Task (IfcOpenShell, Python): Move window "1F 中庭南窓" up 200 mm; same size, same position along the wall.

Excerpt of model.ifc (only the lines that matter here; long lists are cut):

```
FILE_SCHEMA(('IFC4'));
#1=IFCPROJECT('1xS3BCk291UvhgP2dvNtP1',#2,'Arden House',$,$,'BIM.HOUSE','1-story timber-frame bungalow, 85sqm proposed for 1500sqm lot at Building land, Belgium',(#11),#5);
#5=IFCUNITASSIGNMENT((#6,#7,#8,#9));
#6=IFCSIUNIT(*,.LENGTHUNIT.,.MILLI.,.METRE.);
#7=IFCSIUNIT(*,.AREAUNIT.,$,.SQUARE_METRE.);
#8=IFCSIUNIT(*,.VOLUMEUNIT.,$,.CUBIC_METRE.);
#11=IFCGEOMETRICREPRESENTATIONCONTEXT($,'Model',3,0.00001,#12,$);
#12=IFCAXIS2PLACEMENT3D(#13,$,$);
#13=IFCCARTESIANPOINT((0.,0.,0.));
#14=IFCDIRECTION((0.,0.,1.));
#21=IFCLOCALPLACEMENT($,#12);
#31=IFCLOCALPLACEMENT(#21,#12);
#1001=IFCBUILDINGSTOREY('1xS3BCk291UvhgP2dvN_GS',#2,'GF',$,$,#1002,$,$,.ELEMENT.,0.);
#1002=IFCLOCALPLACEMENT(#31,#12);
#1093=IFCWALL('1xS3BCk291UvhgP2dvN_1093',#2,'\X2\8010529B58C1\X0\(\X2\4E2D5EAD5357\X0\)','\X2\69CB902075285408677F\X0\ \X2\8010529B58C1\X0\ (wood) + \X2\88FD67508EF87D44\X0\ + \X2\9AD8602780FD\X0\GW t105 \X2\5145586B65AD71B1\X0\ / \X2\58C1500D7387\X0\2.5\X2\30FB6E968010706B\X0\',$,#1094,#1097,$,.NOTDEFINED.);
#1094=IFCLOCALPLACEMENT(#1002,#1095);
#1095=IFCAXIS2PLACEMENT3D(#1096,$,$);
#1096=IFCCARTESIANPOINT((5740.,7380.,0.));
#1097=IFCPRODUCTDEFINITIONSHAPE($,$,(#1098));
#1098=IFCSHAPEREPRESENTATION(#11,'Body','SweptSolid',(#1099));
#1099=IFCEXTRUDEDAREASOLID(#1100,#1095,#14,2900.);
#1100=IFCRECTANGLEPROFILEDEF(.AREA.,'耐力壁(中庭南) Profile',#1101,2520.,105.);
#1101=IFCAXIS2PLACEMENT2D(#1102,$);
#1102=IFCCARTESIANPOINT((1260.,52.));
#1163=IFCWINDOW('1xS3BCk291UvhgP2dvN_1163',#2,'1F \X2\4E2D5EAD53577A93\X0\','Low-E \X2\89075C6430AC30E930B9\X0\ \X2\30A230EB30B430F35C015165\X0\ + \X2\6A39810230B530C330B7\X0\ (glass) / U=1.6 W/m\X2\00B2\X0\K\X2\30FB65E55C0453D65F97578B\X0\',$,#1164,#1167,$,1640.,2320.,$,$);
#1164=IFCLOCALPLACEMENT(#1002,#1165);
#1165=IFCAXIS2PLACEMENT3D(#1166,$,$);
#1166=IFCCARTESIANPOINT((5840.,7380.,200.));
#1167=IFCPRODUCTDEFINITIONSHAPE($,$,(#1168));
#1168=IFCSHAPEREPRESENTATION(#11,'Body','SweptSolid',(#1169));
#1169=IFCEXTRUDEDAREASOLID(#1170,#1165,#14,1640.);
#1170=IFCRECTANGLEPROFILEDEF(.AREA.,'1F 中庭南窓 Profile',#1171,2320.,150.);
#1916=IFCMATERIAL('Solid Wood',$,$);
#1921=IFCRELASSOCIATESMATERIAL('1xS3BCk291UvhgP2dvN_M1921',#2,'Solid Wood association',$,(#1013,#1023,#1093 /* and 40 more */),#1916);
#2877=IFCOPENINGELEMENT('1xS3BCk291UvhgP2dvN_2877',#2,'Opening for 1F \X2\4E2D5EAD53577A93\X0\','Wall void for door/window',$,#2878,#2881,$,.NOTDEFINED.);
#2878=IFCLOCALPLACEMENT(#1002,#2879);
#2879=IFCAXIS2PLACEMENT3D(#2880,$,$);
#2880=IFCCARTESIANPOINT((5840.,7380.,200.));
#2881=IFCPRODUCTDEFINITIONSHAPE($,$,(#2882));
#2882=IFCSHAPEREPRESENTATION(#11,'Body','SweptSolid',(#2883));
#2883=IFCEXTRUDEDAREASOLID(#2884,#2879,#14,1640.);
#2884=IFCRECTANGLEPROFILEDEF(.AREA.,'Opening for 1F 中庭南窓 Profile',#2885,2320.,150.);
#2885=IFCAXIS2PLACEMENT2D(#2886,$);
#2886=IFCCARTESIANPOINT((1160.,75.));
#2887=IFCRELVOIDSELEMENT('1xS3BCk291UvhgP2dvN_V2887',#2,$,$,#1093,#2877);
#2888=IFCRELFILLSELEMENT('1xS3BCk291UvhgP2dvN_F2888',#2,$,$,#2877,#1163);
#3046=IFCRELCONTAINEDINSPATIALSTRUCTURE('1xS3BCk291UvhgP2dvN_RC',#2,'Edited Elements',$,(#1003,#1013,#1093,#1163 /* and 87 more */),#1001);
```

```python
import numpy as np
import ifcopenshell
import ifcopenshell.api.geometry
import ifcopenshell.util.placement
import ifcopenshell.util.unit

model = ifcopenshell.open("model.ifc")
unit_scale = ifcopenshell.util.unit.calculate_unit_scale(model)

window = model.by_guid("1xS3BCk291UvhgP2dvN_1163")
opening = window.FillsVoids[0].RelatingOpeningElement
dz = 200.0

shift = np.array([0.0, 0.0, dz])
# The window is not placed relative to its opening, so move both.
for product in (opening, window):
    matrix = ifcopenshell.util.placement.get_local_placement(product.ObjectPlacement)
    matrix[:3, 3] += shift
    ifcopenshell.api.geometry.edit_object_placement(model, product=product, matrix=matrix, is_si=False)

print(f"moved by {dz * unit_scale:+.3f} m")

model.write("model-out.ifc")
```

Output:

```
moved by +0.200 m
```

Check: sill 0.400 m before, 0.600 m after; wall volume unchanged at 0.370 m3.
